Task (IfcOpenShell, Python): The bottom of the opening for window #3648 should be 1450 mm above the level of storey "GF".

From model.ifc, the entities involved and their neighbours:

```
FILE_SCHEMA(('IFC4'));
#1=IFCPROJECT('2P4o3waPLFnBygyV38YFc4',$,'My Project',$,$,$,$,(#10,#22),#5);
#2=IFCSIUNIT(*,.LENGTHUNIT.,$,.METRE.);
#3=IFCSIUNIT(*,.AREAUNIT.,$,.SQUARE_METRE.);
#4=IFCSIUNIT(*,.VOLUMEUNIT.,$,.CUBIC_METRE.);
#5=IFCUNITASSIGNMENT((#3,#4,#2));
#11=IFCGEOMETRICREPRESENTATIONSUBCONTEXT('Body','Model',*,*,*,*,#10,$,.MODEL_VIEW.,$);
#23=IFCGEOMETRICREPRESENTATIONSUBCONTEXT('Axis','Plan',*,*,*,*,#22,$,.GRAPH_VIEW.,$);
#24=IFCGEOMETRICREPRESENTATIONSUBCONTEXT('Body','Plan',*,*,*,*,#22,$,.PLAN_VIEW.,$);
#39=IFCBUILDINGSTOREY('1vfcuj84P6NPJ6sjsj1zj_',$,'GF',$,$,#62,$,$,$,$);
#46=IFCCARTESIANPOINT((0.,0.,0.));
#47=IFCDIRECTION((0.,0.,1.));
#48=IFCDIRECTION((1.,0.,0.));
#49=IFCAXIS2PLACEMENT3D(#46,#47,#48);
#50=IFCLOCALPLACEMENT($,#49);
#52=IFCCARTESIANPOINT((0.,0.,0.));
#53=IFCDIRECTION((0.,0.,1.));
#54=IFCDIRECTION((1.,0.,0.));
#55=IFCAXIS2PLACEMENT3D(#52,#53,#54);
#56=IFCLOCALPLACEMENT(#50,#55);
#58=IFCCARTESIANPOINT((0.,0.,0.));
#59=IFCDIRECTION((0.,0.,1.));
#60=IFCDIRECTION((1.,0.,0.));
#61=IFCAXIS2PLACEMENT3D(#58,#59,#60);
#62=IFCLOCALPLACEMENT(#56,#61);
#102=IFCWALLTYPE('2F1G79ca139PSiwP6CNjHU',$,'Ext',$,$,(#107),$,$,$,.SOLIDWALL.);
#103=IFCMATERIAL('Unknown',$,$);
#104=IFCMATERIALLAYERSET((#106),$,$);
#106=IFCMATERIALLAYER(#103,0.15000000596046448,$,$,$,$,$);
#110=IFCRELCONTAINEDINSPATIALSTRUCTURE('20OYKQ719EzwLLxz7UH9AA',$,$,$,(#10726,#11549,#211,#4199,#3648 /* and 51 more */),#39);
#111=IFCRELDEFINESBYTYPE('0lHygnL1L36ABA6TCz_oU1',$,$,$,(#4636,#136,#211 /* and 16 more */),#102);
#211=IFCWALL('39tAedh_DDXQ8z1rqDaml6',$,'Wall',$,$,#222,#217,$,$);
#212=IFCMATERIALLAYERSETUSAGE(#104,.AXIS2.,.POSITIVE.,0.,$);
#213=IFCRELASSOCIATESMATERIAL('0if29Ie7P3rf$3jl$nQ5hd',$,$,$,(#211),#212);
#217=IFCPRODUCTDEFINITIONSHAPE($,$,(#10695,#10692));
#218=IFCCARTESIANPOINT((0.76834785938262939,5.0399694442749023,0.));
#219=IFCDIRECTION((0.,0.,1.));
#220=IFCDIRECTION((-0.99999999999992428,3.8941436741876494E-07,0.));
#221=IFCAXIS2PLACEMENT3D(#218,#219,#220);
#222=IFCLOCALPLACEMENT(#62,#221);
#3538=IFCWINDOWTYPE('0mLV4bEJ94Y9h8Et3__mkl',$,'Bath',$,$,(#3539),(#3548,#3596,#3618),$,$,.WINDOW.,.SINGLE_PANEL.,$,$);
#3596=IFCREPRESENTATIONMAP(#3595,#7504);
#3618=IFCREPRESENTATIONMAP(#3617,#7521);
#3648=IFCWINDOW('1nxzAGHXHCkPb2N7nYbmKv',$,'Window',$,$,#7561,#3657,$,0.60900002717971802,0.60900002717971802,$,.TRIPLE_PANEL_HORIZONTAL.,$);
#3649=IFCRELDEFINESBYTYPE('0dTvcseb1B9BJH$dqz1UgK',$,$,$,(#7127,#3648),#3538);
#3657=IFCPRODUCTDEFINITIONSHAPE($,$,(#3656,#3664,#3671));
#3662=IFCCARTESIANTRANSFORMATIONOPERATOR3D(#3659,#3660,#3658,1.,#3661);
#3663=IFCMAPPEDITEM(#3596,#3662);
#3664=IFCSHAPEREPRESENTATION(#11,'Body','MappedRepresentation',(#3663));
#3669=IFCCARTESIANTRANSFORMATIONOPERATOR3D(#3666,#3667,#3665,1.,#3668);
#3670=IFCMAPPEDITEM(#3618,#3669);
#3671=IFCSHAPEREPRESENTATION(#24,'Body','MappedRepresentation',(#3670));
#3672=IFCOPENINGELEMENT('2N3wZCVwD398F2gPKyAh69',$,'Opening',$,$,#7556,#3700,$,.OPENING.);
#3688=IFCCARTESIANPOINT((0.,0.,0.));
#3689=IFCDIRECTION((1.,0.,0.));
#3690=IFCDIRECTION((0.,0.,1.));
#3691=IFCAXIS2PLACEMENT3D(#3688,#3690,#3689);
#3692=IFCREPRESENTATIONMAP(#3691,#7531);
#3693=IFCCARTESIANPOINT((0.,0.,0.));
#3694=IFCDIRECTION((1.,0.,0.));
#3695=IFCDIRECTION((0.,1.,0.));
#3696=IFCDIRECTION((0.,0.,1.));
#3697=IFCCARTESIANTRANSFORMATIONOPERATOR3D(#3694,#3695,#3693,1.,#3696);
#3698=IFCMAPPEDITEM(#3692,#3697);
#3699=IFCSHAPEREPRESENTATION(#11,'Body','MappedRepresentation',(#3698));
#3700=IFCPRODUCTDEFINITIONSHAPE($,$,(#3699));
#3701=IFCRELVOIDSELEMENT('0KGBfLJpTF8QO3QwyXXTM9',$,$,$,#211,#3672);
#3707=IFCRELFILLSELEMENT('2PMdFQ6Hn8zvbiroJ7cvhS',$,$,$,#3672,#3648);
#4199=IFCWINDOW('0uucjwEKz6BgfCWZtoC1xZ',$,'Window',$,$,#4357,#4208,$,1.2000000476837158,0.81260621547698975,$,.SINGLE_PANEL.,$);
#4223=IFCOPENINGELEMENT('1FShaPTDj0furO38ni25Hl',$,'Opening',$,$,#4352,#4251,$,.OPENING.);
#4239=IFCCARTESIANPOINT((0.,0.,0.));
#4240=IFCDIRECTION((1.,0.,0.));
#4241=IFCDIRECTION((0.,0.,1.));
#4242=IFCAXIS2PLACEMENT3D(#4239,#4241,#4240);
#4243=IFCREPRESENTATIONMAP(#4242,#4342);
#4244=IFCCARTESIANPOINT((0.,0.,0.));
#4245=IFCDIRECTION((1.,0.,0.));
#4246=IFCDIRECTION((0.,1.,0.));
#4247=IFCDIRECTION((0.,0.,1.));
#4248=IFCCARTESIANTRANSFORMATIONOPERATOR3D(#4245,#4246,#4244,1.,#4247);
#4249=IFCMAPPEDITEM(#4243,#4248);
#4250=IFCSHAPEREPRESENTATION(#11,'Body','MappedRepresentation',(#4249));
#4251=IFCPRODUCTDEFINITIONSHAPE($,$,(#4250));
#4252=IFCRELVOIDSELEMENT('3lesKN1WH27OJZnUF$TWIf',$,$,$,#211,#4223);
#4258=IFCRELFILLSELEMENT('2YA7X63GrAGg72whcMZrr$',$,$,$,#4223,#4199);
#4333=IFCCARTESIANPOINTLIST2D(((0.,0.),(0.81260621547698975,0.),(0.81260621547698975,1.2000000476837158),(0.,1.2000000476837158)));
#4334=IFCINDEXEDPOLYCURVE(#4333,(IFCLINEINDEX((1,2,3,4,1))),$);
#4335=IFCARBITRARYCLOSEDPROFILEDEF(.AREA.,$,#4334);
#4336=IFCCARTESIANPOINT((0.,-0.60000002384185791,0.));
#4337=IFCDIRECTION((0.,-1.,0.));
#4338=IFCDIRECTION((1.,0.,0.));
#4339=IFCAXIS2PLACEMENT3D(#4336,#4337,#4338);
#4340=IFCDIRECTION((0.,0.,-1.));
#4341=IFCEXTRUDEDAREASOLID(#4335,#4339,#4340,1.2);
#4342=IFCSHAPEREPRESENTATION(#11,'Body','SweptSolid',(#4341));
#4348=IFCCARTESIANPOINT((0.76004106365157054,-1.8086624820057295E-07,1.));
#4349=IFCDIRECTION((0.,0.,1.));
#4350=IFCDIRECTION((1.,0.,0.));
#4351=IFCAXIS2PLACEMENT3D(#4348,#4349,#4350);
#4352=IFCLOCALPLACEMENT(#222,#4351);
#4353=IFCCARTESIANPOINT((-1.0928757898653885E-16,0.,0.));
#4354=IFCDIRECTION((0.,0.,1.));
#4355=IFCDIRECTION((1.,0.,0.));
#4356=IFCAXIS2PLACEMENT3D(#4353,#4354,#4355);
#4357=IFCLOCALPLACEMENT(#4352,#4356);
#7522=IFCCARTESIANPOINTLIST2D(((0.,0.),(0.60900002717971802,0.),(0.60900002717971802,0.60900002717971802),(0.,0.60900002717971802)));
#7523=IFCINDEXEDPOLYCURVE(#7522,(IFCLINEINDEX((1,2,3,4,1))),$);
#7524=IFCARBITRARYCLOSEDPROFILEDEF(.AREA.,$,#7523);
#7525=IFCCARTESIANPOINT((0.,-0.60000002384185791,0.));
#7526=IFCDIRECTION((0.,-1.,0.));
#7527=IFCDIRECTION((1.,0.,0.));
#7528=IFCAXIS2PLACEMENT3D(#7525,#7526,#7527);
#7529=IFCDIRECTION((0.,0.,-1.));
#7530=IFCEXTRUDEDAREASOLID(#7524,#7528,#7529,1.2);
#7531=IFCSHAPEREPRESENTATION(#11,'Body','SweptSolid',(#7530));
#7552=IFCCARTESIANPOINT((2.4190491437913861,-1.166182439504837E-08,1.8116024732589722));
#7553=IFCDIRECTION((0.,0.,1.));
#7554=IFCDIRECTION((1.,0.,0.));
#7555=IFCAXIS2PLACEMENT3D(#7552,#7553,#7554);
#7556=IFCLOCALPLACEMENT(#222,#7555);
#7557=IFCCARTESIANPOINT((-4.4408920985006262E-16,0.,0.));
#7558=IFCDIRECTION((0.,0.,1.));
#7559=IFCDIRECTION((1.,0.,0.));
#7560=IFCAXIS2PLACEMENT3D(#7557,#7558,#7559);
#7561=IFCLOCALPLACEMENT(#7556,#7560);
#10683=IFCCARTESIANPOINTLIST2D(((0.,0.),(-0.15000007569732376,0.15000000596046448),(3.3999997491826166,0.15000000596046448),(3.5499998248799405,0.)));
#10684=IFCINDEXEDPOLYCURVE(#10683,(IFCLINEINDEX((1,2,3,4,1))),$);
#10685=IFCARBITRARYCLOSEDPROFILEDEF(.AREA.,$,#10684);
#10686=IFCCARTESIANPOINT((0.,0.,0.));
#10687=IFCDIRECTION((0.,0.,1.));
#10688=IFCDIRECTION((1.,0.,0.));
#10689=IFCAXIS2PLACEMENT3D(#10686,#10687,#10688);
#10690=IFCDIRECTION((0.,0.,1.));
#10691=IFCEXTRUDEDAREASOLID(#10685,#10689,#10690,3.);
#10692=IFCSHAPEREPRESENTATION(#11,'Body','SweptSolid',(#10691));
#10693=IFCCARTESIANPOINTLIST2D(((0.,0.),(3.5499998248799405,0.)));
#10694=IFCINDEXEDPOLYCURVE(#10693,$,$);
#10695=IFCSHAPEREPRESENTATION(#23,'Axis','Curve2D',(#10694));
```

```python
import numpy as np
import ifcopenshell
import ifcopenshell.api.geometry
import ifcopenshell.geom
import ifcopenshell.util.element
import ifcopenshell.util.placement
import ifcopenshell.util.shape
import ifcopenshell.util.unit

model = ifcopenshell.open("model.ifc")
unit_scale = ifcopenshell.util.unit.calculate_unit_scale(model)

window = model.by_guid("1nxzAGHXHCkPb2N7nYbmKv")
opening = window.FillsVoids[0].RelatingOpeningElement
storey = ifcopenshell.util.element.get_container(window, ifc_class="IfcBuildingStorey")
level = ifcopenshell.util.placement.get_local_placement(storey.ObjectPlacement)[2, 3]

# The opening's origin need not be at the sill, so measure its lowest point.
shape = ifcopenshell.geom.create_shape(ifcopenshell.geom.settings(), opening)
bottom = ifcopenshell.util.shape.get_shape_bottom_elevation(shape, shape.geometry) / unit_scale
dz = level + 1.45 - bottom

shift = np.array([0.0, 0.0, dz])
# The window is placed relative to its opening, so it follows when the opening moves.
matrix = ifcopenshell.util.placement.get_local_placement(opening.ObjectPlacement)
matrix[:3, 3] += shift
ifcopenshell.api.geometry.edit_object_placement(
    model, product=opening, matrix=matrix, is_si=False, should_transform_children=True
)

print(f"moved by {dz * unit_scale:+.3f} m")

model.write("model_rev.ifc")
```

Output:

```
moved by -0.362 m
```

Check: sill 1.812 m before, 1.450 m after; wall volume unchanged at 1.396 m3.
